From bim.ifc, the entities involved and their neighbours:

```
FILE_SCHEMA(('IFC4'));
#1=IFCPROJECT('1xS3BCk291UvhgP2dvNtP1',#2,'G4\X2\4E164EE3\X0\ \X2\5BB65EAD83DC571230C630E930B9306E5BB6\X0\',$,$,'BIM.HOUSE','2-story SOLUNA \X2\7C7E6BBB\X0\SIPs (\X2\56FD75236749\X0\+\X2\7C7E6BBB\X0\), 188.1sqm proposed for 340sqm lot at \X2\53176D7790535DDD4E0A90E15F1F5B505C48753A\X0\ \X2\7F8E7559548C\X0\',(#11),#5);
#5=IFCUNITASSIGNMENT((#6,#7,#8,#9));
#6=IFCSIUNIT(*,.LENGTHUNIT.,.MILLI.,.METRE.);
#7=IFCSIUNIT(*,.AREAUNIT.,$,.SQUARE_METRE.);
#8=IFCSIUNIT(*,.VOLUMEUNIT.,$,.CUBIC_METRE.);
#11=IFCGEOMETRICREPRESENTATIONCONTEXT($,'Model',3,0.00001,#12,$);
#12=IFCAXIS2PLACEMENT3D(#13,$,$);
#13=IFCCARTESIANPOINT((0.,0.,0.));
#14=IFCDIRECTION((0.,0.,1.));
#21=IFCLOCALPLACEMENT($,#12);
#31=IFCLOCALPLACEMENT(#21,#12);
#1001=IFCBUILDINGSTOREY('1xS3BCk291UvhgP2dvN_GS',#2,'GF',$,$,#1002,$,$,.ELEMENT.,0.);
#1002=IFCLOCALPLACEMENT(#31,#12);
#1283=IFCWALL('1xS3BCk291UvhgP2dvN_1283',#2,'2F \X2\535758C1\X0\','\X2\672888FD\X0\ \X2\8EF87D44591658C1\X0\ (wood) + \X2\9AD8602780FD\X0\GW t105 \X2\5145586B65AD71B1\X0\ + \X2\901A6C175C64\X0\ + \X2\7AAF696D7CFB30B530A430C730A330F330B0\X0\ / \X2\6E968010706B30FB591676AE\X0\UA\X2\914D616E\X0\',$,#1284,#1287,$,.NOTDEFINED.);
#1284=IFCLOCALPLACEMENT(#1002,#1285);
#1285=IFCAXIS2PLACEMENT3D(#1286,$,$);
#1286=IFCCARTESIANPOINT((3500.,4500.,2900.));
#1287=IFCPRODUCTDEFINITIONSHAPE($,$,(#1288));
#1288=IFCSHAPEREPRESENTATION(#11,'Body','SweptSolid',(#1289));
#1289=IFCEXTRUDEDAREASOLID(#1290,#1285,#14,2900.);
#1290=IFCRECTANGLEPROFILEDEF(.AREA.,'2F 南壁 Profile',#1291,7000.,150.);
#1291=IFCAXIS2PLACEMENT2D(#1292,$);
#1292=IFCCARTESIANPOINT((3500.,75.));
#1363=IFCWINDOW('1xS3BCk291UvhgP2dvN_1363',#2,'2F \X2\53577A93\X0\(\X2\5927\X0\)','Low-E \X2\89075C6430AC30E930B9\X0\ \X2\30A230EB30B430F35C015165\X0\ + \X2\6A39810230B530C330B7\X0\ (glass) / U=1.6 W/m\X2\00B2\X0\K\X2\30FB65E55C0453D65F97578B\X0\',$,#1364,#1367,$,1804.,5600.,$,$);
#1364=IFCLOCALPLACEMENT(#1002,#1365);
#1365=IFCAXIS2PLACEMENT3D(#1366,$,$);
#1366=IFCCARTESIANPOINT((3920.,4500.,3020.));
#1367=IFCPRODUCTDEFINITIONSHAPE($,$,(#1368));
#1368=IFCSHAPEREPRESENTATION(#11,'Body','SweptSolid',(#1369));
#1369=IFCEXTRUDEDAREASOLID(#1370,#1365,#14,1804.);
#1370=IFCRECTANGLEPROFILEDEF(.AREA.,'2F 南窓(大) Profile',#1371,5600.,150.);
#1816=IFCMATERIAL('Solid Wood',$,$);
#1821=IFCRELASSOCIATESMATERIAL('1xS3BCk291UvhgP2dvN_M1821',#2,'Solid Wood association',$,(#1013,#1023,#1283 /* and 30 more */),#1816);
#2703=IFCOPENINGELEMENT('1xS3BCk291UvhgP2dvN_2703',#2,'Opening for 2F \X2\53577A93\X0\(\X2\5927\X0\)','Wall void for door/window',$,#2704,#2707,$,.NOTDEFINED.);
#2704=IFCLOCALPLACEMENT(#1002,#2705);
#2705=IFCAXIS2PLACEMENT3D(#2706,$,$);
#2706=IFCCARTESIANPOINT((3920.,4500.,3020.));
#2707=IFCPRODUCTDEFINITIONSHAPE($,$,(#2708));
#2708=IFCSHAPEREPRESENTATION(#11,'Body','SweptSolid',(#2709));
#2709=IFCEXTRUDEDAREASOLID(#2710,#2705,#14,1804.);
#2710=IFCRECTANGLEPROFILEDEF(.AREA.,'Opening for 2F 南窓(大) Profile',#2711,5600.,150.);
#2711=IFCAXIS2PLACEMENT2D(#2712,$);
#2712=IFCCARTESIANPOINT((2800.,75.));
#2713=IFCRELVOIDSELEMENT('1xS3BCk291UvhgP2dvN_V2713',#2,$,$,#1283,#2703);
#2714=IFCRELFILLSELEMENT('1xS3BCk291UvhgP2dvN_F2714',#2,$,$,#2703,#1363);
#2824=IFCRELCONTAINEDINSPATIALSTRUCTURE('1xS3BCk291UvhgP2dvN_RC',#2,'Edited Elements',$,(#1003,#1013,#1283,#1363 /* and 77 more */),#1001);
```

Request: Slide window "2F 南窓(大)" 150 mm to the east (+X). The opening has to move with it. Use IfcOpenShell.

```python
import ifcopenshell
import ifcopenshell.api.geometry
import ifcopenshell.util.placement
import ifcopenshell.util.unit

model = ifcopenshell.open("bim.ifc")
unit_scale = ifcopenshell.util.unit.calculate_unit_scale(model)

window = model.by_id(1363)
opening = window.FillsVoids[0].RelatingOpeningElement
wall = opening.VoidsElements[0].RelatingBuildingElement

wall_matrix = ifcopenshell.util.placement.get_local_placement(wall.ObjectPlacement)
shift = wall_matrix[:3, 0] * 0.15 / unit_scale
before = ifcopenshell.util.placement.get_local_placement(window.ObjectPlacement)[:3, 3].copy()

# The window is not placed relative to its opening, so move both.
for product in (opening, window):
    matrix = ifcopenshell.util.placement.get_local_placement(product.ObjectPlacement)
    matrix[:3, 3] += shift
    ifcopenshell.api.geometry.edit_object_placement(model, product=product, matrix=matrix, is_si=False)

after = ifcopenshell.util.placement.get_local_placement(window.ObjectPlacement)[:3, 3]
print("window moved by", (after - before).round(3) + 0.0)

model.write("bim_updated.ifc")
```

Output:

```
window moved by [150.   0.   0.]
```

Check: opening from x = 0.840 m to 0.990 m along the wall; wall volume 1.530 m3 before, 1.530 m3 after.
